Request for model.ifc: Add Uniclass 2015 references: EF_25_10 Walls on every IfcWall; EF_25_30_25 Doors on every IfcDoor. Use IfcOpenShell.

First a look at what the model holds.

```python
import ifcopenshell

model = ifcopenshell.open("model.ifc")
print(model.schema)
print("classifications:", [c.Name for c in model.by_type("IfcClassification")])
for ifc_class in ("IfcDoor", "IfcRoof", "IfcStair", "IfcWall", "IfcWindow"):
    print(ifc_class, len(model.by_type(ifc_class)))
```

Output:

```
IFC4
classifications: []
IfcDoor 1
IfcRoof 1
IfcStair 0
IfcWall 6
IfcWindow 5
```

```python
import ifcopenshell
import ifcopenshell.api.classification

model = ifcopenshell.open("model.ifc")

system = ifcopenshell.api.classification.add_classification(model, classification="Uniclass 2015")

codes = {
    "IfcWall": ("EF_25_10", "Walls"),
    "IfcDoor": ("EF_25_30_25", "Doors"),
}
for ifc_class, (code, name) in codes.items():
    products = model.by_type(ifc_class)
    ifcopenshell.api.classification.add_reference(
        model, products=products, classification=system, identification=code, name=name
    )
    print(code, len(products))

model.write("model_edited.ifc")
```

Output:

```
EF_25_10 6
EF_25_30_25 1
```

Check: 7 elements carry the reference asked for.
